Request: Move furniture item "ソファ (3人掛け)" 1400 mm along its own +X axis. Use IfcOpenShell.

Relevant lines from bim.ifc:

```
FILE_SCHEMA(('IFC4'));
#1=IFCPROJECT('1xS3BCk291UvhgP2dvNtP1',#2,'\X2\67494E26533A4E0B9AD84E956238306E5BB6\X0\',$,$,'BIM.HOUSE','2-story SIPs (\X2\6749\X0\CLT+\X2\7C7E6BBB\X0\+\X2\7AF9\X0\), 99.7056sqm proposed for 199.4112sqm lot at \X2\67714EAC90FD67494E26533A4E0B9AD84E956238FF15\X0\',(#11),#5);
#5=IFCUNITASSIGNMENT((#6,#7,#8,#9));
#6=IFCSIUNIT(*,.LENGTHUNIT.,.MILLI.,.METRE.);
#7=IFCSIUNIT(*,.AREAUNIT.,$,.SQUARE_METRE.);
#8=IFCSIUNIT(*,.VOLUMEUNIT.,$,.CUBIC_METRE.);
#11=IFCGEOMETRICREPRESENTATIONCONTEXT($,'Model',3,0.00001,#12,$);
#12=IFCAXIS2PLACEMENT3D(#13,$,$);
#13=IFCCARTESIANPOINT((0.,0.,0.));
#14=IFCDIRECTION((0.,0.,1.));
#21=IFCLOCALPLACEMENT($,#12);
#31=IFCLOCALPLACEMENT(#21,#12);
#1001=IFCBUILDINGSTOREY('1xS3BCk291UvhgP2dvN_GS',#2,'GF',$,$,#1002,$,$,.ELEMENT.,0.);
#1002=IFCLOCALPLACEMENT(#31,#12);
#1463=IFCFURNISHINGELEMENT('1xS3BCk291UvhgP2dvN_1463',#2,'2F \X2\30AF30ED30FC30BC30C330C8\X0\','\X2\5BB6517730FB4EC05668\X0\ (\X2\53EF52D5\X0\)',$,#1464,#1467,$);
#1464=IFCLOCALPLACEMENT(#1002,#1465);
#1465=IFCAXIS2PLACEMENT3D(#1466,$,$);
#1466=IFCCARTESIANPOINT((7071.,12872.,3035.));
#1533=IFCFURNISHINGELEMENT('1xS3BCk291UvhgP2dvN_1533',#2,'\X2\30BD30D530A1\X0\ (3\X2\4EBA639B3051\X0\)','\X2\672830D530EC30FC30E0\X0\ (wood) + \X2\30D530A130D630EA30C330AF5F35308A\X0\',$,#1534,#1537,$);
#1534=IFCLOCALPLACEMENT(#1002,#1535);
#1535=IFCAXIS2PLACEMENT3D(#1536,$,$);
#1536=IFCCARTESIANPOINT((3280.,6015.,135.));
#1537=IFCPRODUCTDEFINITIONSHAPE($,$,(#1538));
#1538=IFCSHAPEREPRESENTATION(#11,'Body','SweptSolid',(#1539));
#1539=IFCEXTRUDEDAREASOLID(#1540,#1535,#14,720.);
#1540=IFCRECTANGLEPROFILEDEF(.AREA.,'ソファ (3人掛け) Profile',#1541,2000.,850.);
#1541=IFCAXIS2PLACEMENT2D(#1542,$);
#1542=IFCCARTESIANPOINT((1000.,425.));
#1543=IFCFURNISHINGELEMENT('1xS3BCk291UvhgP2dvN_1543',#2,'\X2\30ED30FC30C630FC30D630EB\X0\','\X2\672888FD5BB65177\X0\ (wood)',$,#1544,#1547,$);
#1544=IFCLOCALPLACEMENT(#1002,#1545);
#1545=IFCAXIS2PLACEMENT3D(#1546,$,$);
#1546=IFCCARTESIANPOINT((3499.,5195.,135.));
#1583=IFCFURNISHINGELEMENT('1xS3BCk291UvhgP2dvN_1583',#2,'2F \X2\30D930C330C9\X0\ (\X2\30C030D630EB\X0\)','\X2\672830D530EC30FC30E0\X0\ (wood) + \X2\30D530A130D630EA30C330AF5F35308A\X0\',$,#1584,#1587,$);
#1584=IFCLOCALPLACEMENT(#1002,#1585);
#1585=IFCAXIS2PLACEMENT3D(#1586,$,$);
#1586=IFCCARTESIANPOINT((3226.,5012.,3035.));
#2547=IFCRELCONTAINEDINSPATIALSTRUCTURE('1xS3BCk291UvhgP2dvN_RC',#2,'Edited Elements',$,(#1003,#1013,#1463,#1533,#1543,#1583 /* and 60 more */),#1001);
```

```python
import ifcopenshell
import ifcopenshell.api.geometry
import ifcopenshell.util.placement
import ifcopenshell.util.unit

model = ifcopenshell.open("bim.ifc")
unit_scale = ifcopenshell.util.unit.calculate_unit_scale(model)

item = model.by_id(1533)
matrix = ifcopenshell.util.placement.get_local_placement(item.ObjectPlacement)
matrix[:3, 3] += matrix[:3, 0] * 1.4 / unit_scale
ifcopenshell.api.geometry.edit_object_placement(model, product=item, matrix=matrix, is_si=False)

print(ifcopenshell.util.placement.get_local_placement(item.ObjectPlacement).round(3) + 0.0)

model.write("bim_updated.ifc")
```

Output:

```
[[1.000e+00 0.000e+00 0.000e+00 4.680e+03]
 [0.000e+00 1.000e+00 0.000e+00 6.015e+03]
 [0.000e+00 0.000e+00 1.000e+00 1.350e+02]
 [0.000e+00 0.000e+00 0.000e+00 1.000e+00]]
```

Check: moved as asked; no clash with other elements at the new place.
